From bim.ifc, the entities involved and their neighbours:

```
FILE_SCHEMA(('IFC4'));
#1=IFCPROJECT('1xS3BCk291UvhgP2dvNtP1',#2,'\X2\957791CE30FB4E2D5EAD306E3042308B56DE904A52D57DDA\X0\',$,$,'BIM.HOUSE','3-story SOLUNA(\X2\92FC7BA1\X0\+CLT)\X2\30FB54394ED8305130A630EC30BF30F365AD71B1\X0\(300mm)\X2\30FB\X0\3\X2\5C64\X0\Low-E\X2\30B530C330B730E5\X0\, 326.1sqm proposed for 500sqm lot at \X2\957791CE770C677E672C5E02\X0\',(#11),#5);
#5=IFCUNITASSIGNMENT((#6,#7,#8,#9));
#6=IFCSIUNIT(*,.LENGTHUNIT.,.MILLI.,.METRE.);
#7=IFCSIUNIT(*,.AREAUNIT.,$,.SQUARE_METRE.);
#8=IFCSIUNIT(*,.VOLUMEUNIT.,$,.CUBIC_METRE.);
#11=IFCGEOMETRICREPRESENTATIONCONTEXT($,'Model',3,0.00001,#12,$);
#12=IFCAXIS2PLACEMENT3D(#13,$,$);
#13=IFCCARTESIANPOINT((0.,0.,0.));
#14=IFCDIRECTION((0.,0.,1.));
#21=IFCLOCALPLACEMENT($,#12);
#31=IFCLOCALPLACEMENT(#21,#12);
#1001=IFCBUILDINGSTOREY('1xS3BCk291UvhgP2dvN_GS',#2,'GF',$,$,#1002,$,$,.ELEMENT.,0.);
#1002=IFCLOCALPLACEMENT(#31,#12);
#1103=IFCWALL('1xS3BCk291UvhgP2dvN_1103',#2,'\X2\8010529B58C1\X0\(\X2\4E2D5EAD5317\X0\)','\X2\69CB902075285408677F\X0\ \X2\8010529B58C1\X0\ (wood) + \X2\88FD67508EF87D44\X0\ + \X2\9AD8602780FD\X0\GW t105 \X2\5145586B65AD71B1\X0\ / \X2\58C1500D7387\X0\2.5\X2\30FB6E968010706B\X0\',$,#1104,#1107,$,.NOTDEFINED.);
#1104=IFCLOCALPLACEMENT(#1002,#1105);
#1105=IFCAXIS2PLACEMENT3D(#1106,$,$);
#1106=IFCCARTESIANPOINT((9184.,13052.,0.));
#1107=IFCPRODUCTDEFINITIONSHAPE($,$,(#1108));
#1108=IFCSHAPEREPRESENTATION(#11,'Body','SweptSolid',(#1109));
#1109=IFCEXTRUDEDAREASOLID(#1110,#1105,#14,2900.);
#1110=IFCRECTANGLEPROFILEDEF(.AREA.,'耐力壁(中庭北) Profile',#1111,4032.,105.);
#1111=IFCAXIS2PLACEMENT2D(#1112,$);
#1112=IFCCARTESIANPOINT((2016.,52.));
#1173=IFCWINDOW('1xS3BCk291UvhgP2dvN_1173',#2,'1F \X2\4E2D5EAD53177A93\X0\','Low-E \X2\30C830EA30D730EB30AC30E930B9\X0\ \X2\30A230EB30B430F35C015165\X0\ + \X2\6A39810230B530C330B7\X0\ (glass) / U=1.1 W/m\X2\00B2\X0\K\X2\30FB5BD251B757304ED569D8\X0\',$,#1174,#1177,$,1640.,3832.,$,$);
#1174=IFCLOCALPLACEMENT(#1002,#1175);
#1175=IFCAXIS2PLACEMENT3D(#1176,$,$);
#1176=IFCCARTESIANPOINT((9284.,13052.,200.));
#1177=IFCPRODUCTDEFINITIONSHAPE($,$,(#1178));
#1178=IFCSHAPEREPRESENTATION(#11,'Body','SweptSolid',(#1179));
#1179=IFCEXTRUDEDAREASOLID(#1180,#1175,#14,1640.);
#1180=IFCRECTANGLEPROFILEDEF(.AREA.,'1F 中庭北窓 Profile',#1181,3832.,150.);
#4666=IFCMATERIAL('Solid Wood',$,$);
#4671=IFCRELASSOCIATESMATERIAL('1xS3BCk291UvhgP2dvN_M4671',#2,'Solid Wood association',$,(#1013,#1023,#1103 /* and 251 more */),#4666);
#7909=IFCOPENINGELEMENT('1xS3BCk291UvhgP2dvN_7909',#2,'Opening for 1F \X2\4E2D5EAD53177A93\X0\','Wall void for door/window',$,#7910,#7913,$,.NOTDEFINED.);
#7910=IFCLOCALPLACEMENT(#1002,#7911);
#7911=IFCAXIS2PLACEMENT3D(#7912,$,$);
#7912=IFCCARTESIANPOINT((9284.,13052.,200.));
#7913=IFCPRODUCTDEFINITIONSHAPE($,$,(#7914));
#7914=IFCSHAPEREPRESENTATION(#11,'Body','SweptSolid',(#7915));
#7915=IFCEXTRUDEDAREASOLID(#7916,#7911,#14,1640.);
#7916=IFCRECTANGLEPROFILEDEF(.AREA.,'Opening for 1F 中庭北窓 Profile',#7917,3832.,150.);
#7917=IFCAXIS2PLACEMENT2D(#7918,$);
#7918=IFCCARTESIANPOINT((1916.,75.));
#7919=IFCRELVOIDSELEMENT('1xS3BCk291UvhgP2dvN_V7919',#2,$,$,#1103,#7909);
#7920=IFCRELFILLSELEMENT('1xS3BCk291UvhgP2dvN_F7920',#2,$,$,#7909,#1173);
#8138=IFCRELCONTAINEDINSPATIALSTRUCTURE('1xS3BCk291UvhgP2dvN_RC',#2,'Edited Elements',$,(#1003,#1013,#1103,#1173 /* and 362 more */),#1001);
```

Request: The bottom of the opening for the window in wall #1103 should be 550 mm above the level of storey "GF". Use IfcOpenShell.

```python
import numpy as np
import ifcopenshell
import ifcopenshell.api.geometry
import ifcopenshell.geom
import ifcopenshell.util.element
import ifcopenshell.util.placement
import ifcopenshell.util.shape
import ifcopenshell.util.unit

model = ifcopenshell.open("bim.ifc")
unit_scale = ifcopenshell.util.unit.calculate_unit_scale(model)

window = model.by_id(1173)
opening = window.FillsVoids[0].RelatingOpeningElement
storey = ifcopenshell.util.element.get_container(window, ifc_class="IfcBuildingStorey")
level = ifcopenshell.util.placement.get_local_placement(storey.ObjectPlacement)[2, 3]

# The opening's origin need not be at the sill, so measure its lowest point.
shape = ifcopenshell.geom.create_shape(ifcopenshell.geom.settings(), opening)
bottom = ifcopenshell.util.shape.get_shape_bottom_elevation(shape, shape.geometry) / unit_scale
dz = level + 0.55 / unit_scale - bottom

shift = np.array([0.0, 0.0, dz])
# The window is not placed relative to its opening, so move both.
for product in (opening, window):
    matrix = ifcopenshell.util.placement.get_local_placement(product.ObjectPlacement)
    matrix[:3, 3] += shift
    ifcopenshell.api.geometry.edit_object_placement(model, product=product, matrix=matrix, is_si=False)

print(f"moved by {dz * unit_scale:+.3f} m")

model.write("bim_rev.ifc")
```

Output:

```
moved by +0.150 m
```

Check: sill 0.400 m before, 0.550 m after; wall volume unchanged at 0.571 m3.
